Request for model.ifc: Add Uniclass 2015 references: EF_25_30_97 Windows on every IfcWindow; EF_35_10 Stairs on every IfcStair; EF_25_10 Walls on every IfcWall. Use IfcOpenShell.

First a look at what the model holds.

```python
import ifcopenshell

model = ifcopenshell.open("model.ifc")
print(model.schema)
print("classifications:", [c.Name for c in model.by_type("IfcClassification")])
for ifc_class in ("IfcDoor", "IfcRoof", "IfcStair", "IfcWall", "IfcWindow"):
    print(ifc_class, len(model.by_type(ifc_class)))
```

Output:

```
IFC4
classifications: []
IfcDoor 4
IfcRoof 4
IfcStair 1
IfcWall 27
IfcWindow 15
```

```python
import ifcopenshell
import ifcopenshell.api.classification

model = ifcopenshell.open("model.ifc")

system = ifcopenshell.api.classification.add_classification(model, classification="Uniclass 2015")

codes = {
    "IfcWindow": ("EF_25_30_97", "Windows"),
    "IfcStair": ("EF_35_10", "Stairs"),
    "IfcWall": ("EF_25_10", "Walls"),
}
for ifc_class, (code, name) in codes.items():
    products = model.by_type(ifc_class)
    ifcopenshell.api.classification.add_reference(
        model, products=products, classification=system, identification=code, name=name
    )
    print(code, len(products))

model.write("model_rev.ifc")
```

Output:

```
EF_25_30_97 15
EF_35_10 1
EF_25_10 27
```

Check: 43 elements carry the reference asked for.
